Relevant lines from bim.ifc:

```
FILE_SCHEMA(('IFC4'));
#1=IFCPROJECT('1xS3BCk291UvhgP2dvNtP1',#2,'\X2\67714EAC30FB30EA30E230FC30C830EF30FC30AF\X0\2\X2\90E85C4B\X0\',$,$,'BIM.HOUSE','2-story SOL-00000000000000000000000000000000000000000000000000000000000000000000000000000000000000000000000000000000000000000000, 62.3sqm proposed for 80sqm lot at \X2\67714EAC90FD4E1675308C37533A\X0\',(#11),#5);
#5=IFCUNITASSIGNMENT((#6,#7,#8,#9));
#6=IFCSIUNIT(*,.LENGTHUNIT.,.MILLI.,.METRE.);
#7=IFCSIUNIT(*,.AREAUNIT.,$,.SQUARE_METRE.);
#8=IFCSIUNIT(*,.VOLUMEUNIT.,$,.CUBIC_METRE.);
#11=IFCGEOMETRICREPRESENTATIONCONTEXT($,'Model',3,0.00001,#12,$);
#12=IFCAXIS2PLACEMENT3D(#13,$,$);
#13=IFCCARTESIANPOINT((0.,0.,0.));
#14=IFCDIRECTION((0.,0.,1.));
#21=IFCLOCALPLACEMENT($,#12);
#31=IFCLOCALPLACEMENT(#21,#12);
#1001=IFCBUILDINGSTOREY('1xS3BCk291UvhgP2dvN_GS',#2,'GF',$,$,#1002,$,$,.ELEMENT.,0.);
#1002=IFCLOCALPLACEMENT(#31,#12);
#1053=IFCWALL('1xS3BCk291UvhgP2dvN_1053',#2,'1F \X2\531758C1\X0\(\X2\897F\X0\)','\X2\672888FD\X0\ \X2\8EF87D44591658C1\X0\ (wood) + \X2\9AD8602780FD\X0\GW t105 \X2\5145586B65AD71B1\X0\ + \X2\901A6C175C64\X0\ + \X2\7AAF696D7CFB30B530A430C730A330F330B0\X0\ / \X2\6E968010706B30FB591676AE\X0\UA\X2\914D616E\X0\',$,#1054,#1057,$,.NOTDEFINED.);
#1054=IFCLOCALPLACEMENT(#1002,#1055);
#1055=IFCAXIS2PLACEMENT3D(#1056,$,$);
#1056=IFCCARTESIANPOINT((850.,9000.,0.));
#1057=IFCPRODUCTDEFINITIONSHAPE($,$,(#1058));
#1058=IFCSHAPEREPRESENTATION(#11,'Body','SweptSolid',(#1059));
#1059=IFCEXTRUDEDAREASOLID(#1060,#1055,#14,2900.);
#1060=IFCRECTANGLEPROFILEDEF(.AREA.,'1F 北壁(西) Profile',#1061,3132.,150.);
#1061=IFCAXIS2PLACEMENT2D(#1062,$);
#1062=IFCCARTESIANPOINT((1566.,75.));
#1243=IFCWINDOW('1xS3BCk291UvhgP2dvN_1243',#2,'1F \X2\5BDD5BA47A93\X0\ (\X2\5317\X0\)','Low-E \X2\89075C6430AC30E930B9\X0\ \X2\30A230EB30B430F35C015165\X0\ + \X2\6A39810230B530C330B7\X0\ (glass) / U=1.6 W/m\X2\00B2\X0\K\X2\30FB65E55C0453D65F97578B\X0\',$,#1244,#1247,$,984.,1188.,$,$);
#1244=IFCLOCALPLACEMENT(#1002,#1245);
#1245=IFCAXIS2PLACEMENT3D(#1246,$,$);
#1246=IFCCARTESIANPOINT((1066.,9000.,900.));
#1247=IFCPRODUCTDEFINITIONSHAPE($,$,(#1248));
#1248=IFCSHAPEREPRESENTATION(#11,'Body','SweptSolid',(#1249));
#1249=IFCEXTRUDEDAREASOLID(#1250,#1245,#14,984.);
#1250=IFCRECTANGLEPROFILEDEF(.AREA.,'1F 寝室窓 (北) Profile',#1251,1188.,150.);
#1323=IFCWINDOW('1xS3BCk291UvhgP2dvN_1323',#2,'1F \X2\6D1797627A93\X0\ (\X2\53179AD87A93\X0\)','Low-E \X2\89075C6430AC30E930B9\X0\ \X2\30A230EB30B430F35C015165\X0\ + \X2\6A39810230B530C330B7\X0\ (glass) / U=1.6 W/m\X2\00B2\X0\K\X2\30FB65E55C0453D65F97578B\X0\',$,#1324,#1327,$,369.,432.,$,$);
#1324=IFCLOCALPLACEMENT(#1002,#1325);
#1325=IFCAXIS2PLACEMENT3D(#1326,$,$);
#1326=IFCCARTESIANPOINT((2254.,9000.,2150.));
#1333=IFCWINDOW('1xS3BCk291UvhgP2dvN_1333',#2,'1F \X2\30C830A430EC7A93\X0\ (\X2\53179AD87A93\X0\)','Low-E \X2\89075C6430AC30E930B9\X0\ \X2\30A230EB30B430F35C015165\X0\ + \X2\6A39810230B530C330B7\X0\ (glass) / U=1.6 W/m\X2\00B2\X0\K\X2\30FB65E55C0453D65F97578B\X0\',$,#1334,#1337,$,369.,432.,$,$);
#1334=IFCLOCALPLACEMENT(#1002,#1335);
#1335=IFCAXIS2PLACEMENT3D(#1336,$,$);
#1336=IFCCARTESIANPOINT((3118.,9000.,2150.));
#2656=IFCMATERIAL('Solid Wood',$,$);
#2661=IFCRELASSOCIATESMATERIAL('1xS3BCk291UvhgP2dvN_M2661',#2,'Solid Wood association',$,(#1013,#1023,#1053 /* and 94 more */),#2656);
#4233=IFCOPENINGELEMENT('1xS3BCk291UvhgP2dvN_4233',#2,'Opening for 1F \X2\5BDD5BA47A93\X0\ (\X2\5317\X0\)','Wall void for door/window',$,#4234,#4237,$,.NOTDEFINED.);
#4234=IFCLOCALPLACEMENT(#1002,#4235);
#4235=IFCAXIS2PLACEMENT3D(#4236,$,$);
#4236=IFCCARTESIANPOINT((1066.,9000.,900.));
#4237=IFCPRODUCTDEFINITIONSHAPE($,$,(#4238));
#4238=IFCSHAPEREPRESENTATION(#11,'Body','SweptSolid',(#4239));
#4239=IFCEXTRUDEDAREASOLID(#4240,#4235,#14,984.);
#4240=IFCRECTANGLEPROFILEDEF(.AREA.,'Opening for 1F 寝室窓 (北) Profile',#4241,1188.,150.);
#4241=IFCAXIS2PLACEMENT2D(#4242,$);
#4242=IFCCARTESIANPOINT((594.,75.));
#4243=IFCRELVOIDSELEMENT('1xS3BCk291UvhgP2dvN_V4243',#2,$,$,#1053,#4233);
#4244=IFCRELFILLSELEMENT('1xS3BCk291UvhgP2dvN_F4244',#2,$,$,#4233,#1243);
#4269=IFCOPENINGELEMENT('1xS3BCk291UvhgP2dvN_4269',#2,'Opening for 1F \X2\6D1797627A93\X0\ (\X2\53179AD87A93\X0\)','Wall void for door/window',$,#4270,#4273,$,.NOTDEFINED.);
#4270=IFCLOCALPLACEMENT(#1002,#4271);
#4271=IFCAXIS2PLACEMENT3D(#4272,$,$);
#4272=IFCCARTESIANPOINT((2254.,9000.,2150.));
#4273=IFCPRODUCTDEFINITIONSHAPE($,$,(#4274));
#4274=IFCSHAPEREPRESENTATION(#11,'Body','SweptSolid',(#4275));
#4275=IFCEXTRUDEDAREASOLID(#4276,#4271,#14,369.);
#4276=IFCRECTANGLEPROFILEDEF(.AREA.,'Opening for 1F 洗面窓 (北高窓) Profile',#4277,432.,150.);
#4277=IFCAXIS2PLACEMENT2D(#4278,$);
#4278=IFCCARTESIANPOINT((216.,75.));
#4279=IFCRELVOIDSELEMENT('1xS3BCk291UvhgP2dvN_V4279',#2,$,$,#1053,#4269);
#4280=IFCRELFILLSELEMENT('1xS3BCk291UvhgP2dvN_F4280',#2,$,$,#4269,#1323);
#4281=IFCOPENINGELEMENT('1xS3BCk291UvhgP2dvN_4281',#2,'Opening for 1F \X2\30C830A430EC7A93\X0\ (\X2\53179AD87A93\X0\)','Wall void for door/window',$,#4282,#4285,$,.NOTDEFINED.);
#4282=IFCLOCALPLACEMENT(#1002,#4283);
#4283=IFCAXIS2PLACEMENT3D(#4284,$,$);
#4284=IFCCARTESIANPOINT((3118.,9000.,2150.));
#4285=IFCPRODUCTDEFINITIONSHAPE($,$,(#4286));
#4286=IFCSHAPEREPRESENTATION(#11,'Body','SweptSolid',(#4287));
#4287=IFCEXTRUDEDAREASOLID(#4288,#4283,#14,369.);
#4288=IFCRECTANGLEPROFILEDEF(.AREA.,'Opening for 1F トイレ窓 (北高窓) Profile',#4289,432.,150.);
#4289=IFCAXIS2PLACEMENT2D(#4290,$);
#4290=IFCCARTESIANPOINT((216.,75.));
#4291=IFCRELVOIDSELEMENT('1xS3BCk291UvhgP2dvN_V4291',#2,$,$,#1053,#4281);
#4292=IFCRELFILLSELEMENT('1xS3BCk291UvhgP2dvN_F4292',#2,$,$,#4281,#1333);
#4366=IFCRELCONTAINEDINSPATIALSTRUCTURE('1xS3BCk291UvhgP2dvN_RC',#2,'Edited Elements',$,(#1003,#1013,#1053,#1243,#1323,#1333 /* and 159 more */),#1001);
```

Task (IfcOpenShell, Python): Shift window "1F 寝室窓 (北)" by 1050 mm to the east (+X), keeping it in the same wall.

```python
import ifcopenshell
import ifcopenshell.api.geometry
import ifcopenshell.util.placement
import ifcopenshell.util.unit

model = ifcopenshell.open("bim.ifc")
unit_scale = ifcopenshell.util.unit.calculate_unit_scale(model)

window = model.by_guid("1xS3BCk291UvhgP2dvN_1243")
opening = window.FillsVoids[0].RelatingOpeningElement
wall = opening.VoidsElements[0].RelatingBuildingElement

wall_matrix = ifcopenshell.util.placement.get_local_placement(wall.ObjectPlacement)
shift = wall_matrix[:3, 0] * 1.05 / unit_scale
before = ifcopenshell.util.placement.get_local_placement(window.ObjectPlacement)[:3, 3].copy()

# The window is not placed relative to its opening, so move both.
for product in (opening, window):
    matrix = ifcopenshell.util.placement.get_local_placement(product.ObjectPlacement)
    matrix[:3, 3] += shift
    ifcopenshell.api.geometry.edit_object_placement(model, product=product, matrix=matrix, is_si=False)

after = ifcopenshell.util.placement.get_local_placement(window.ObjectPlacement)[:3, 3]
print("window moved by", (after - before).round(3) + 0.0)

model.write("bim-out.ifc")
```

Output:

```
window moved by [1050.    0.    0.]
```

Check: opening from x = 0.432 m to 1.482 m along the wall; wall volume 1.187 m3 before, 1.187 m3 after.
